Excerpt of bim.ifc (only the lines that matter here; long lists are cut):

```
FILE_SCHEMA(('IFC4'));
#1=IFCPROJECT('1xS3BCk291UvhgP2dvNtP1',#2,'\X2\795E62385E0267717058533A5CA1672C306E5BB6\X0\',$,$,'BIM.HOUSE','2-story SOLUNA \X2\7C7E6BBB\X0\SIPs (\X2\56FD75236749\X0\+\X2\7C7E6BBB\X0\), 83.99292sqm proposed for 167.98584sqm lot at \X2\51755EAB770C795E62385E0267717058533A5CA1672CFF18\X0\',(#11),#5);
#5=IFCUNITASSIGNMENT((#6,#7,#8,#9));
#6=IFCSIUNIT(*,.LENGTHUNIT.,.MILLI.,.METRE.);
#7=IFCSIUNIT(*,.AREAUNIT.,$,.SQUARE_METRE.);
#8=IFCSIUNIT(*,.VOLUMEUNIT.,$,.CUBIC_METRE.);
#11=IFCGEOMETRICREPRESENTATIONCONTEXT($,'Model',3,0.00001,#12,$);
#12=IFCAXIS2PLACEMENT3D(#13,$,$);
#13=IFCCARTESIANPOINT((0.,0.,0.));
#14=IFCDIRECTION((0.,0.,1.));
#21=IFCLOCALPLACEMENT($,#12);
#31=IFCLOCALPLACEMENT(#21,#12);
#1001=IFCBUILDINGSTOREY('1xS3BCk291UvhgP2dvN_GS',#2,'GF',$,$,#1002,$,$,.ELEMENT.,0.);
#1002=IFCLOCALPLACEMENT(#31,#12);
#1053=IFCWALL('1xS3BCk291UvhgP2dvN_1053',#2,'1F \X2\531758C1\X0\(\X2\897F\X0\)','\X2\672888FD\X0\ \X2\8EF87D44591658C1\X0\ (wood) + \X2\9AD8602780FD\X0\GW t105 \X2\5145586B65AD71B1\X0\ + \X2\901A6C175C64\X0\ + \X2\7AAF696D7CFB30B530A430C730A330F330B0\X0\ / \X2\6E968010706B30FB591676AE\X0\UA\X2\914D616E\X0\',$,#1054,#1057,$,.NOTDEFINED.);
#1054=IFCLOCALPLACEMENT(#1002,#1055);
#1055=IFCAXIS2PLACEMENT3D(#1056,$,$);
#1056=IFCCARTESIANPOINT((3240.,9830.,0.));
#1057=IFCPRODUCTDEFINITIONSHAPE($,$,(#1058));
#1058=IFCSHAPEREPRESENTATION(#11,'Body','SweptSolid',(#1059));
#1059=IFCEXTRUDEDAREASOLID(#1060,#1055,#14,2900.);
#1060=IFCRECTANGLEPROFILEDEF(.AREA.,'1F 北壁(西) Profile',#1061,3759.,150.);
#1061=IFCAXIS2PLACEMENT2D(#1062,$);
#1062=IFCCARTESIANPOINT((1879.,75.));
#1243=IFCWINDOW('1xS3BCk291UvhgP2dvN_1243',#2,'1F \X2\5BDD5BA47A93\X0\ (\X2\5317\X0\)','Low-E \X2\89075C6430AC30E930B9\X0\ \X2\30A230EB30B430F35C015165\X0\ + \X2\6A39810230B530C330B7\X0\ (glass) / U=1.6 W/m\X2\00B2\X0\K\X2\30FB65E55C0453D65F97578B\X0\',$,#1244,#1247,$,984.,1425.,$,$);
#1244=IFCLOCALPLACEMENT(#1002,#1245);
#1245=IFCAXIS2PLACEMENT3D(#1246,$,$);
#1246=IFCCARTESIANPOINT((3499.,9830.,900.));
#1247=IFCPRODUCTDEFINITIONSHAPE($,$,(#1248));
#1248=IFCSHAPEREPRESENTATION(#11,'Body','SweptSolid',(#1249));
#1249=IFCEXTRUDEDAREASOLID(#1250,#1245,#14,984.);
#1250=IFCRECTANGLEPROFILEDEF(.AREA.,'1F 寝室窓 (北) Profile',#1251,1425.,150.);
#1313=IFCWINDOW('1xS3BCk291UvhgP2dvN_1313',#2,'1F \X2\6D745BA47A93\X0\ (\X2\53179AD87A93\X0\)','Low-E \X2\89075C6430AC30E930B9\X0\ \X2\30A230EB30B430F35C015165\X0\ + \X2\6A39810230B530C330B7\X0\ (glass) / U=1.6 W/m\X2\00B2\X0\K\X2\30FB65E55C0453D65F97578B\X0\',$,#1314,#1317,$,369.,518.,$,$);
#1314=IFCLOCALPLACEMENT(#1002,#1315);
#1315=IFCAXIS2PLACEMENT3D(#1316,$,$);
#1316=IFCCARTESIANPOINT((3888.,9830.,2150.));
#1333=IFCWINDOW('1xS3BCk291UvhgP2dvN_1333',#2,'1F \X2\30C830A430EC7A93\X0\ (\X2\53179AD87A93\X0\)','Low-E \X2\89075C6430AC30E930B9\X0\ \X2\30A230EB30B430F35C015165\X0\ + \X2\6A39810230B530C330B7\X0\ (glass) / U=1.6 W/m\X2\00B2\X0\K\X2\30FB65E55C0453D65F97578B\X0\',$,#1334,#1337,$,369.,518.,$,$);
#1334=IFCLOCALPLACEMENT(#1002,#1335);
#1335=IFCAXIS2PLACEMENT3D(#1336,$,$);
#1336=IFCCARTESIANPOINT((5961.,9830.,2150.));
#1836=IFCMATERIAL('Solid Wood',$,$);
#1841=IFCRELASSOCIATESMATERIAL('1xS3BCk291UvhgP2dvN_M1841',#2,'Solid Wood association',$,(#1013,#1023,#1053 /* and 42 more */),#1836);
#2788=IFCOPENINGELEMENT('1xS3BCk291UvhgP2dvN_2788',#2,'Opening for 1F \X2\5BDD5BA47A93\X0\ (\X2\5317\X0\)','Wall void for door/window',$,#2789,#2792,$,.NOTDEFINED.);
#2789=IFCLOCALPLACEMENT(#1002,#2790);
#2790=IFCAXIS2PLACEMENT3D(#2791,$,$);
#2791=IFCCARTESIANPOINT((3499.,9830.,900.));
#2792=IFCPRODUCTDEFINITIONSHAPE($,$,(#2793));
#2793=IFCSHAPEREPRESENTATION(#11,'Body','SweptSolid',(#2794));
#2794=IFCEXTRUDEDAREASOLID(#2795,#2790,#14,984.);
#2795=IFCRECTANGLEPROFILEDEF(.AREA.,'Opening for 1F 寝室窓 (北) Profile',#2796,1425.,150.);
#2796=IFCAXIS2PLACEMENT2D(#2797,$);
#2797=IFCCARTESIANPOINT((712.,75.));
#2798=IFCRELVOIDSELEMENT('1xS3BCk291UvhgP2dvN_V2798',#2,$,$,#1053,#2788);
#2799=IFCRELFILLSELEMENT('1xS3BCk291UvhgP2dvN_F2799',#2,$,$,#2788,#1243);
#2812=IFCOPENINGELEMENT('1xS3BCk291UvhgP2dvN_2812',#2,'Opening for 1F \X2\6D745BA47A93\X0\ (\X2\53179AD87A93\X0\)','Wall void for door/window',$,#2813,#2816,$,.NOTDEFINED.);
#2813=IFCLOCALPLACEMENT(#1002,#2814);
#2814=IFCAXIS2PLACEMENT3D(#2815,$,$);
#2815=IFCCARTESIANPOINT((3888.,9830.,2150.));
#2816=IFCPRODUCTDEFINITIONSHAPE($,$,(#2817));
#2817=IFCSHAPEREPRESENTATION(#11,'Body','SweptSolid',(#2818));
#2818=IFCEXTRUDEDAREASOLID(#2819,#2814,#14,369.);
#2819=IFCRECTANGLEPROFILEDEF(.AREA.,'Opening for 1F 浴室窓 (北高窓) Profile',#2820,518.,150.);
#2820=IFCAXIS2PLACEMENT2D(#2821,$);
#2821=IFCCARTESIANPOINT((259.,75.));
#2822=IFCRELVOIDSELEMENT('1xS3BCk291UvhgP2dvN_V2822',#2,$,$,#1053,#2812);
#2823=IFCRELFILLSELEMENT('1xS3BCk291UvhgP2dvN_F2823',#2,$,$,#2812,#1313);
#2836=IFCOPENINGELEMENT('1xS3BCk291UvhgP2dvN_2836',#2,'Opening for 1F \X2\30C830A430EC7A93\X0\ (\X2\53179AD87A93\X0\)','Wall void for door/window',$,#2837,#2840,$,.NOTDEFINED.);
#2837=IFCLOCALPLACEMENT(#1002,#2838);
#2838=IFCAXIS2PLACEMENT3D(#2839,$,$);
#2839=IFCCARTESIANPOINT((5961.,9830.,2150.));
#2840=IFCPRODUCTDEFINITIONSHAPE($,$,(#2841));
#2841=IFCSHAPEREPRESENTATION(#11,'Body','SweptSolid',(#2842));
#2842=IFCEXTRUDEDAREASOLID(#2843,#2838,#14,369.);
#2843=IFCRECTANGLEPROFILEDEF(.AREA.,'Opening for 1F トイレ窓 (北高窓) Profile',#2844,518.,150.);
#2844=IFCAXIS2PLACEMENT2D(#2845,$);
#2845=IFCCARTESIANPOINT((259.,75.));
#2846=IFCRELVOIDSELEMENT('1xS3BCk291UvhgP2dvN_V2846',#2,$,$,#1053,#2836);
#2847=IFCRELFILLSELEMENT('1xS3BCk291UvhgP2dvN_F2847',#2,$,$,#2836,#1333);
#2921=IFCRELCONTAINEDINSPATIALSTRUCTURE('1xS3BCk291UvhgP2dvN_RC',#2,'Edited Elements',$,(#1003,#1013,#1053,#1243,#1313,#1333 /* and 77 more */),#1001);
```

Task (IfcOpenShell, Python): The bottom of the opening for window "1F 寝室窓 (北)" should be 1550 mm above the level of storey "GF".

```python
import numpy as np
import ifcopenshell
import ifcopenshell.api.geometry
import ifcopenshell.geom
import ifcopenshell.util.element
import ifcopenshell.util.placement
import ifcopenshell.util.shape
import ifcopenshell.util.unit

model = ifcopenshell.open("bim.ifc")
unit_scale = ifcopenshell.util.unit.calculate_unit_scale(model)

window = model.by_guid("1xS3BCk291UvhgP2dvN_1243")
opening = window.FillsVoids[0].RelatingOpeningElement
storey = ifcopenshell.util.element.get_container(window, ifc_class="IfcBuildingStorey")
level = ifcopenshell.util.placement.get_local_placement(storey.ObjectPlacement)[2, 3]

# The opening's origin need not be at the sill, so measure its lowest point.
shape = ifcopenshell.geom.create_shape(ifcopenshell.geom.settings(), opening)
bottom = ifcopenshell.util.shape.get_shape_bottom_elevation(shape, shape.geometry) / unit_scale
dz = level + 1.55 / unit_scale - bottom

shift = np.array([0.0, 0.0, dz])
# The window is not placed relative to its opening, so move both.
for product in (opening, window):
    matrix = ifcopenshell.util.placement.get_local_placement(product.ObjectPlacement)
    matrix[:3, 3] += shift
    ifcopenshell.api.geometry.edit_object_placement(model, product=product, matrix=matrix, is_si=False)

print(f"moved by {dz * unit_scale:+.3f} m")

model.write("bim-out.ifc")
```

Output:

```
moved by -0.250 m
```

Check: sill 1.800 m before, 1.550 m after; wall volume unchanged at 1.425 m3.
